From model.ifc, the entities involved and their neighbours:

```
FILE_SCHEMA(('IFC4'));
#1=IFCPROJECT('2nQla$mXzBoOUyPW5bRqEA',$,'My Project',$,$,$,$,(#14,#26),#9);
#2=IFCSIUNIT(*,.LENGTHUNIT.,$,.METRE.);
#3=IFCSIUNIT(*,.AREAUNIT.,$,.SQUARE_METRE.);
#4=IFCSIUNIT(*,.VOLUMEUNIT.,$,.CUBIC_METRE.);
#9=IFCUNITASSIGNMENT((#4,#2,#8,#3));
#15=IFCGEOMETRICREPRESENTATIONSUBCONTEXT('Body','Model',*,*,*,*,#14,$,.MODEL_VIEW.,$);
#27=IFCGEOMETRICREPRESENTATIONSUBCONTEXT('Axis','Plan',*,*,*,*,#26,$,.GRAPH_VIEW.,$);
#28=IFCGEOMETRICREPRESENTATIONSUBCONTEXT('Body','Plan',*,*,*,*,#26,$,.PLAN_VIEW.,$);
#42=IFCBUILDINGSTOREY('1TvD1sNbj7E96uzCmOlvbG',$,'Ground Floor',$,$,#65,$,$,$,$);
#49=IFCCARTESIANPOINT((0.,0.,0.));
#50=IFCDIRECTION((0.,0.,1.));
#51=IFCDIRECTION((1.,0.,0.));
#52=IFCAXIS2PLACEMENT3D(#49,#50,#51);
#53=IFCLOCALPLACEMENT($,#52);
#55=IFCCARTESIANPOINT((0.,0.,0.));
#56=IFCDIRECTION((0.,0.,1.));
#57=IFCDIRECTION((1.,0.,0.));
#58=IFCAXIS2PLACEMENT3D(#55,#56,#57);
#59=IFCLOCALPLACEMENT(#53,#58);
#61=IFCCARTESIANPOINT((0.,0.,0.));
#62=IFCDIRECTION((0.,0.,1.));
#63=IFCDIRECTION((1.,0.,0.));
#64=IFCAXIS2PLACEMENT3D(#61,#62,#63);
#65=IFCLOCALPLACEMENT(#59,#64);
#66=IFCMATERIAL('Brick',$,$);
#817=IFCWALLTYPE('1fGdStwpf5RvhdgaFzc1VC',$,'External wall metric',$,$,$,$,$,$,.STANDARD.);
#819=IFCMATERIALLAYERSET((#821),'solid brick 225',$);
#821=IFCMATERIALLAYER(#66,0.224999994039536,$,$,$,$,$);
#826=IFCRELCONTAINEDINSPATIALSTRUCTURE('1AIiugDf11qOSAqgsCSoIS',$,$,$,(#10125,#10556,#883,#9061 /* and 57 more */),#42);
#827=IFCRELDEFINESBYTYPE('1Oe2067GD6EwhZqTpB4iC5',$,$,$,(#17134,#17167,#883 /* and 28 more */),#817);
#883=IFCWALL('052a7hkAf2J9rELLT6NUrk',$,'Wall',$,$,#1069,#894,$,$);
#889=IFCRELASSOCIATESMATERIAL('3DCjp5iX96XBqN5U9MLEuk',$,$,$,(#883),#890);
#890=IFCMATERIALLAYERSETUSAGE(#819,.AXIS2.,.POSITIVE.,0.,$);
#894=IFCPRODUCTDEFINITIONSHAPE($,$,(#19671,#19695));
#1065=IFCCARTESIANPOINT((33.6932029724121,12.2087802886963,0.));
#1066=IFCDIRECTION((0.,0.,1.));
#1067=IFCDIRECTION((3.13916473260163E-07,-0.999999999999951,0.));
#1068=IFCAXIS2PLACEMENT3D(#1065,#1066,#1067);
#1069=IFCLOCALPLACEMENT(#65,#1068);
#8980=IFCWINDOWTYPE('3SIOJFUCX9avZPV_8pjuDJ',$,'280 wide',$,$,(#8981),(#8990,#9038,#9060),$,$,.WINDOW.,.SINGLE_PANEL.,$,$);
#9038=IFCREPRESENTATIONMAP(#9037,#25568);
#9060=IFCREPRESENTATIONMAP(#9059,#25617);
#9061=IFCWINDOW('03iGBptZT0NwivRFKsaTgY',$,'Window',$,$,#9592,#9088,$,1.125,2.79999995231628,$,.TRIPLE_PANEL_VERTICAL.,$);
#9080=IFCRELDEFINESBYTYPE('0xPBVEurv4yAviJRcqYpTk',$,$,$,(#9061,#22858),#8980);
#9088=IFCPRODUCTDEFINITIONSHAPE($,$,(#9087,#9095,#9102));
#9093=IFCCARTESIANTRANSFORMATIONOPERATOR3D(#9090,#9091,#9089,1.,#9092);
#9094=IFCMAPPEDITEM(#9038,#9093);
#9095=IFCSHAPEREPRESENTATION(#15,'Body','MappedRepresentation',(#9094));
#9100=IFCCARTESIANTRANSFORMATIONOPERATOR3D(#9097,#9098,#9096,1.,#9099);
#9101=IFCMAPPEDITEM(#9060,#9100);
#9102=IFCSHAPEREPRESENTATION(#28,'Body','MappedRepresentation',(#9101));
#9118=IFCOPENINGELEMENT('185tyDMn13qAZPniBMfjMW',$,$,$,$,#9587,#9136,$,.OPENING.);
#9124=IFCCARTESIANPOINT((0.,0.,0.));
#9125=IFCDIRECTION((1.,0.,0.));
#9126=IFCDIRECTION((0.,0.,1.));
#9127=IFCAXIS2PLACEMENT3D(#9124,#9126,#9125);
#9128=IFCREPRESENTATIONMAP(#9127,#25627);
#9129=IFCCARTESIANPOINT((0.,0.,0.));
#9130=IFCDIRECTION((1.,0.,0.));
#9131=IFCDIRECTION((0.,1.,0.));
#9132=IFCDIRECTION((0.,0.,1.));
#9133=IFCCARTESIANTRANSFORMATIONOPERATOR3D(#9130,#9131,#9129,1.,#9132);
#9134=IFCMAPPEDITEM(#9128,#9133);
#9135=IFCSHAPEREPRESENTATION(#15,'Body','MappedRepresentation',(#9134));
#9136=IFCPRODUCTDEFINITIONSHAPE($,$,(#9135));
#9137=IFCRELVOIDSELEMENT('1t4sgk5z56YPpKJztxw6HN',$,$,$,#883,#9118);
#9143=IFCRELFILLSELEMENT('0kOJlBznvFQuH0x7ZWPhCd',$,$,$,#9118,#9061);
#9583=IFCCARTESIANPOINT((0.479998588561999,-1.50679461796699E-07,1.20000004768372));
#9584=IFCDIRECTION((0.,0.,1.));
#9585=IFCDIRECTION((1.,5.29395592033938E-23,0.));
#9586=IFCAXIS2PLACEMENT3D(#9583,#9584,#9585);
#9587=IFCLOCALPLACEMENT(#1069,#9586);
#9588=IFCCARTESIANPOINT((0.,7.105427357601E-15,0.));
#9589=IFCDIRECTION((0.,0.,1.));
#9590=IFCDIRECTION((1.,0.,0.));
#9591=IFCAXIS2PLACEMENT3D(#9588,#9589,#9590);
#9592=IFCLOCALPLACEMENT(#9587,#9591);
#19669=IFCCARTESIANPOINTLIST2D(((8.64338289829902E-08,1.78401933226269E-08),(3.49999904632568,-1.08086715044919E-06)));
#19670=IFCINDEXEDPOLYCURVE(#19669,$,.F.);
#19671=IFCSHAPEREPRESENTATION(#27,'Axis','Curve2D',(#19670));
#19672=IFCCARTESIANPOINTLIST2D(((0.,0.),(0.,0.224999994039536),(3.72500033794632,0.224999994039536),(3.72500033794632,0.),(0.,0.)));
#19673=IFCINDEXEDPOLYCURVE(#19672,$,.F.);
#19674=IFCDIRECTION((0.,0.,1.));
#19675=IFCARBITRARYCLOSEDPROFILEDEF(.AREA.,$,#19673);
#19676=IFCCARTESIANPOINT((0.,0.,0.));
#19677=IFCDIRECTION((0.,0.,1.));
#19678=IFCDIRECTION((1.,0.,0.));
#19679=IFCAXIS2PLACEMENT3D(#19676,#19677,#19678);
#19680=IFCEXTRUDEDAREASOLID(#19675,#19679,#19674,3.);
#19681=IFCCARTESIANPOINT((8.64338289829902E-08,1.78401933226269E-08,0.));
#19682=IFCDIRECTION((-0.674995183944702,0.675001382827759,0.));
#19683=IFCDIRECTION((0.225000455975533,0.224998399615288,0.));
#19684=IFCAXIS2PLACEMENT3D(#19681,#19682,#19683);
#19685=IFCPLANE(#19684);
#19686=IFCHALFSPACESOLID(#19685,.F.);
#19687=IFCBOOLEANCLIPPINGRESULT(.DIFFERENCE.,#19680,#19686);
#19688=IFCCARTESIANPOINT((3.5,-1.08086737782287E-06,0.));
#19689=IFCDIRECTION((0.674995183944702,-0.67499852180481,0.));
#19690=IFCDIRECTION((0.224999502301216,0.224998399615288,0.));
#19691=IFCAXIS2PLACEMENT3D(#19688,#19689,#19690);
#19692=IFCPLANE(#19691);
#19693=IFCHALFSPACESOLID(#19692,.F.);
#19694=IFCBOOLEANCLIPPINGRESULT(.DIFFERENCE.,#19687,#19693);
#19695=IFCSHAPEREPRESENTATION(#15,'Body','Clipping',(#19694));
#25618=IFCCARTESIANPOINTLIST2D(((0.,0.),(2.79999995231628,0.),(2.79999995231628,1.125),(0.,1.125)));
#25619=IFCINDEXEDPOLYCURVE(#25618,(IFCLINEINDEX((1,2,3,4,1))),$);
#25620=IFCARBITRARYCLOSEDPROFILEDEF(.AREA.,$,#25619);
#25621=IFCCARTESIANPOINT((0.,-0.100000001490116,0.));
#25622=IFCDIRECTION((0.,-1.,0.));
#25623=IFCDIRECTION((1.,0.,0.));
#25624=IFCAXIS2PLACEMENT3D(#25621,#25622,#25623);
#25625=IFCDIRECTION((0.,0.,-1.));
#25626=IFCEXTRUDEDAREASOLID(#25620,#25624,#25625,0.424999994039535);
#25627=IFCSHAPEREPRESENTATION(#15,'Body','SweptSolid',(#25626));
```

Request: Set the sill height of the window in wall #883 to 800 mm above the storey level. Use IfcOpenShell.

```python
import numpy as np
import ifcopenshell
import ifcopenshell.api.geometry
import ifcopenshell.geom
import ifcopenshell.util.element
import ifcopenshell.util.placement
import ifcopenshell.util.shape
import ifcopenshell.util.unit

model = ifcopenshell.open("model.ifc")
unit_scale = ifcopenshell.util.unit.calculate_unit_scale(model)

window = model.by_guid("03iGBptZT0NwivRFKsaTgY")
opening = window.FillsVoids[0].RelatingOpeningElement
storey = ifcopenshell.util.element.get_container(window, ifc_class="IfcBuildingStorey")
level = ifcopenshell.util.placement.get_local_placement(storey.ObjectPlacement)[2, 3]

# The opening's origin need not be at the sill, so measure its lowest point.
shape = ifcopenshell.geom.create_shape(ifcopenshell.geom.settings(), opening)
bottom = ifcopenshell.util.shape.get_shape_bottom_elevation(shape, shape.geometry) / unit_scale
dz = level + 0.8 - bottom

shift = np.array([0.0, 0.0, dz])
# The window is placed relative to its opening, so it follows when the opening moves.
matrix = ifcopenshell.util.placement.get_local_placement(opening.ObjectPlacement)
matrix[:3, 3] += shift
ifcopenshell.api.geometry.edit_object_placement(
    model, product=opening, matrix=matrix, is_si=False, should_transform_children=True
)

print(f"moved by {dz * unit_scale:+.3f} m")

model.write("model_updated.ifc")
```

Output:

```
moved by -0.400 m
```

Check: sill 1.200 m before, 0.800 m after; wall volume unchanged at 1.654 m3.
